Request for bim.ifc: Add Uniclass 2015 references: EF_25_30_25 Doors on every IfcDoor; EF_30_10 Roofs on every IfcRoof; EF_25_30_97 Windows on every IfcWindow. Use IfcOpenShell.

First a look at what the model holds.

```python
import ifcopenshell

model = ifcopenshell.open("bim.ifc")
print(model.schema)
print("classifications:", [c.Name for c in model.by_type("IfcClassification")])
for ifc_class in ("IfcDoor", "IfcRoof", "IfcStair", "IfcWall", "IfcWindow"):
    print(ifc_class, len(model.by_type(ifc_class)))
```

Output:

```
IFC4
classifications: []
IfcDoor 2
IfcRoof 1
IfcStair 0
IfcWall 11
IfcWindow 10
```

```python
import ifcopenshell
import ifcopenshell.api.classification

model = ifcopenshell.open("bim.ifc")

system = ifcopenshell.api.classification.add_classification(model, classification="Uniclass 2015")

codes = {
    "IfcDoor": ("EF_25_30_25", "Doors"),
    "IfcRoof": ("EF_30_10", "Roofs"),
    "IfcWindow": ("EF_25_30_97", "Windows"),
}
for ifc_class, (code, name) in codes.items():
    products = model.by_type(ifc_class)
    ifcopenshell.api.classification.add_reference(
        model, products=products, classification=system, identification=code, name=name
    )
    print(code, len(products))

model.write("bim_edited.ifc")
```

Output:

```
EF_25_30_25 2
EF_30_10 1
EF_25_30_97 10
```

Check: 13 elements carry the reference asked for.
